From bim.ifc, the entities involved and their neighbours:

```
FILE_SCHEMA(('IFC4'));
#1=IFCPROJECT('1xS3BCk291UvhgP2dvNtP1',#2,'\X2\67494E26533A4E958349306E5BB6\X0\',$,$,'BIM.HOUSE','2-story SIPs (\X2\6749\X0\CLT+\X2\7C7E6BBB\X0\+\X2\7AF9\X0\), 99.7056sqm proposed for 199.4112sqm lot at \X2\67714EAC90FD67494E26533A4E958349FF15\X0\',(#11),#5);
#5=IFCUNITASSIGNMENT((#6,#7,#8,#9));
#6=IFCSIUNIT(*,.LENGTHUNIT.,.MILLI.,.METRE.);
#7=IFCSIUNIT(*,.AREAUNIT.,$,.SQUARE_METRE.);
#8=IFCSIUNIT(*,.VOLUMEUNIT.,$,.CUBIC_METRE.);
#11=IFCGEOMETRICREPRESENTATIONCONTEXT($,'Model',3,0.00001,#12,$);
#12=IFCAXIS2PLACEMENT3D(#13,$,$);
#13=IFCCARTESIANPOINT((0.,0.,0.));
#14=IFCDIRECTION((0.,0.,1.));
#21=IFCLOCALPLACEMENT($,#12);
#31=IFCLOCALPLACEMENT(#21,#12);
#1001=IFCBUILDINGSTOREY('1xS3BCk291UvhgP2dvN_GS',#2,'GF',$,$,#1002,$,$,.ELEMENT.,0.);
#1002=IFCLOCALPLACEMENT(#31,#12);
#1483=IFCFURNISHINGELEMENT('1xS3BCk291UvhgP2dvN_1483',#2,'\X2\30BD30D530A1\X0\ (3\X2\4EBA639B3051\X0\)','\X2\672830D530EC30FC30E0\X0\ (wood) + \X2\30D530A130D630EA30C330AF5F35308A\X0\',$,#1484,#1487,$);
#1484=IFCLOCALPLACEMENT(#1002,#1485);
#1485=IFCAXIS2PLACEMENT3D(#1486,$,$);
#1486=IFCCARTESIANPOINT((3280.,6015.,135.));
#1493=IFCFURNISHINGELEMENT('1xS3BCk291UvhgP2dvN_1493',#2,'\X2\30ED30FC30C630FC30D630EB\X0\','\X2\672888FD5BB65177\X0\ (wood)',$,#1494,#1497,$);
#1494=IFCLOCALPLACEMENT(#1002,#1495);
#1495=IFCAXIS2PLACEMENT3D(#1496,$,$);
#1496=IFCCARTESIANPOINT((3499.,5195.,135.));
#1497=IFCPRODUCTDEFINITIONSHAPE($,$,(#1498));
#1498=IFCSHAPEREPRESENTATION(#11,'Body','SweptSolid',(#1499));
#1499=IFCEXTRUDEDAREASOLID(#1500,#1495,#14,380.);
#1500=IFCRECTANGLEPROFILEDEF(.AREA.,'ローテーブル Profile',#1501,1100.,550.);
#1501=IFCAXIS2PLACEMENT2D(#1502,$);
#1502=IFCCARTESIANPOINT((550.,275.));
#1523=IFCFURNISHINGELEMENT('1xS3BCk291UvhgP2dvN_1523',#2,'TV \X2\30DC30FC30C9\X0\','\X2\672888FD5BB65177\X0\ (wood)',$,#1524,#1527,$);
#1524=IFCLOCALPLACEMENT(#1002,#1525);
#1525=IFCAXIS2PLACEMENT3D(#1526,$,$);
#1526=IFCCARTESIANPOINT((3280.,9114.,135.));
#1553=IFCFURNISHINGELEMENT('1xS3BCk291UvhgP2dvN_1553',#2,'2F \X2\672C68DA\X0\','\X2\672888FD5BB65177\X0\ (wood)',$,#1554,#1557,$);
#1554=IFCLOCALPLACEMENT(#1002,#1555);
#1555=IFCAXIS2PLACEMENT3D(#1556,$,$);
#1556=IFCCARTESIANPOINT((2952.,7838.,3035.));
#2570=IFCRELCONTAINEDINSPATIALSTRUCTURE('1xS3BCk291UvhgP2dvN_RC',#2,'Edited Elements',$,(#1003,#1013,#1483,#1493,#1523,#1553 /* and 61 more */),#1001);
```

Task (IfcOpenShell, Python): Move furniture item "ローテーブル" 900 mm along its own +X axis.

```python
import ifcopenshell
import ifcopenshell.api.geometry
import ifcopenshell.util.placement

model = ifcopenshell.open("bim.ifc")

item = model.by_guid("1xS3BCk291UvhgP2dvN_1493")
matrix = ifcopenshell.util.placement.get_local_placement(item.ObjectPlacement)
matrix[:3, 3] += matrix[:3, 0] * 900.0
ifcopenshell.api.geometry.edit_object_placement(model, product=item, matrix=matrix, is_si=False)

print(ifcopenshell.util.placement.get_local_placement(item.ObjectPlacement).round(3) + 0.0)

model.write("bim-out.ifc")
```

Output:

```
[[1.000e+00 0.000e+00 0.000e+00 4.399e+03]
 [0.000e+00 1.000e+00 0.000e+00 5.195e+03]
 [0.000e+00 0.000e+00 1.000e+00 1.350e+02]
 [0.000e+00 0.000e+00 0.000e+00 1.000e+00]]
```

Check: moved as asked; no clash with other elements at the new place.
